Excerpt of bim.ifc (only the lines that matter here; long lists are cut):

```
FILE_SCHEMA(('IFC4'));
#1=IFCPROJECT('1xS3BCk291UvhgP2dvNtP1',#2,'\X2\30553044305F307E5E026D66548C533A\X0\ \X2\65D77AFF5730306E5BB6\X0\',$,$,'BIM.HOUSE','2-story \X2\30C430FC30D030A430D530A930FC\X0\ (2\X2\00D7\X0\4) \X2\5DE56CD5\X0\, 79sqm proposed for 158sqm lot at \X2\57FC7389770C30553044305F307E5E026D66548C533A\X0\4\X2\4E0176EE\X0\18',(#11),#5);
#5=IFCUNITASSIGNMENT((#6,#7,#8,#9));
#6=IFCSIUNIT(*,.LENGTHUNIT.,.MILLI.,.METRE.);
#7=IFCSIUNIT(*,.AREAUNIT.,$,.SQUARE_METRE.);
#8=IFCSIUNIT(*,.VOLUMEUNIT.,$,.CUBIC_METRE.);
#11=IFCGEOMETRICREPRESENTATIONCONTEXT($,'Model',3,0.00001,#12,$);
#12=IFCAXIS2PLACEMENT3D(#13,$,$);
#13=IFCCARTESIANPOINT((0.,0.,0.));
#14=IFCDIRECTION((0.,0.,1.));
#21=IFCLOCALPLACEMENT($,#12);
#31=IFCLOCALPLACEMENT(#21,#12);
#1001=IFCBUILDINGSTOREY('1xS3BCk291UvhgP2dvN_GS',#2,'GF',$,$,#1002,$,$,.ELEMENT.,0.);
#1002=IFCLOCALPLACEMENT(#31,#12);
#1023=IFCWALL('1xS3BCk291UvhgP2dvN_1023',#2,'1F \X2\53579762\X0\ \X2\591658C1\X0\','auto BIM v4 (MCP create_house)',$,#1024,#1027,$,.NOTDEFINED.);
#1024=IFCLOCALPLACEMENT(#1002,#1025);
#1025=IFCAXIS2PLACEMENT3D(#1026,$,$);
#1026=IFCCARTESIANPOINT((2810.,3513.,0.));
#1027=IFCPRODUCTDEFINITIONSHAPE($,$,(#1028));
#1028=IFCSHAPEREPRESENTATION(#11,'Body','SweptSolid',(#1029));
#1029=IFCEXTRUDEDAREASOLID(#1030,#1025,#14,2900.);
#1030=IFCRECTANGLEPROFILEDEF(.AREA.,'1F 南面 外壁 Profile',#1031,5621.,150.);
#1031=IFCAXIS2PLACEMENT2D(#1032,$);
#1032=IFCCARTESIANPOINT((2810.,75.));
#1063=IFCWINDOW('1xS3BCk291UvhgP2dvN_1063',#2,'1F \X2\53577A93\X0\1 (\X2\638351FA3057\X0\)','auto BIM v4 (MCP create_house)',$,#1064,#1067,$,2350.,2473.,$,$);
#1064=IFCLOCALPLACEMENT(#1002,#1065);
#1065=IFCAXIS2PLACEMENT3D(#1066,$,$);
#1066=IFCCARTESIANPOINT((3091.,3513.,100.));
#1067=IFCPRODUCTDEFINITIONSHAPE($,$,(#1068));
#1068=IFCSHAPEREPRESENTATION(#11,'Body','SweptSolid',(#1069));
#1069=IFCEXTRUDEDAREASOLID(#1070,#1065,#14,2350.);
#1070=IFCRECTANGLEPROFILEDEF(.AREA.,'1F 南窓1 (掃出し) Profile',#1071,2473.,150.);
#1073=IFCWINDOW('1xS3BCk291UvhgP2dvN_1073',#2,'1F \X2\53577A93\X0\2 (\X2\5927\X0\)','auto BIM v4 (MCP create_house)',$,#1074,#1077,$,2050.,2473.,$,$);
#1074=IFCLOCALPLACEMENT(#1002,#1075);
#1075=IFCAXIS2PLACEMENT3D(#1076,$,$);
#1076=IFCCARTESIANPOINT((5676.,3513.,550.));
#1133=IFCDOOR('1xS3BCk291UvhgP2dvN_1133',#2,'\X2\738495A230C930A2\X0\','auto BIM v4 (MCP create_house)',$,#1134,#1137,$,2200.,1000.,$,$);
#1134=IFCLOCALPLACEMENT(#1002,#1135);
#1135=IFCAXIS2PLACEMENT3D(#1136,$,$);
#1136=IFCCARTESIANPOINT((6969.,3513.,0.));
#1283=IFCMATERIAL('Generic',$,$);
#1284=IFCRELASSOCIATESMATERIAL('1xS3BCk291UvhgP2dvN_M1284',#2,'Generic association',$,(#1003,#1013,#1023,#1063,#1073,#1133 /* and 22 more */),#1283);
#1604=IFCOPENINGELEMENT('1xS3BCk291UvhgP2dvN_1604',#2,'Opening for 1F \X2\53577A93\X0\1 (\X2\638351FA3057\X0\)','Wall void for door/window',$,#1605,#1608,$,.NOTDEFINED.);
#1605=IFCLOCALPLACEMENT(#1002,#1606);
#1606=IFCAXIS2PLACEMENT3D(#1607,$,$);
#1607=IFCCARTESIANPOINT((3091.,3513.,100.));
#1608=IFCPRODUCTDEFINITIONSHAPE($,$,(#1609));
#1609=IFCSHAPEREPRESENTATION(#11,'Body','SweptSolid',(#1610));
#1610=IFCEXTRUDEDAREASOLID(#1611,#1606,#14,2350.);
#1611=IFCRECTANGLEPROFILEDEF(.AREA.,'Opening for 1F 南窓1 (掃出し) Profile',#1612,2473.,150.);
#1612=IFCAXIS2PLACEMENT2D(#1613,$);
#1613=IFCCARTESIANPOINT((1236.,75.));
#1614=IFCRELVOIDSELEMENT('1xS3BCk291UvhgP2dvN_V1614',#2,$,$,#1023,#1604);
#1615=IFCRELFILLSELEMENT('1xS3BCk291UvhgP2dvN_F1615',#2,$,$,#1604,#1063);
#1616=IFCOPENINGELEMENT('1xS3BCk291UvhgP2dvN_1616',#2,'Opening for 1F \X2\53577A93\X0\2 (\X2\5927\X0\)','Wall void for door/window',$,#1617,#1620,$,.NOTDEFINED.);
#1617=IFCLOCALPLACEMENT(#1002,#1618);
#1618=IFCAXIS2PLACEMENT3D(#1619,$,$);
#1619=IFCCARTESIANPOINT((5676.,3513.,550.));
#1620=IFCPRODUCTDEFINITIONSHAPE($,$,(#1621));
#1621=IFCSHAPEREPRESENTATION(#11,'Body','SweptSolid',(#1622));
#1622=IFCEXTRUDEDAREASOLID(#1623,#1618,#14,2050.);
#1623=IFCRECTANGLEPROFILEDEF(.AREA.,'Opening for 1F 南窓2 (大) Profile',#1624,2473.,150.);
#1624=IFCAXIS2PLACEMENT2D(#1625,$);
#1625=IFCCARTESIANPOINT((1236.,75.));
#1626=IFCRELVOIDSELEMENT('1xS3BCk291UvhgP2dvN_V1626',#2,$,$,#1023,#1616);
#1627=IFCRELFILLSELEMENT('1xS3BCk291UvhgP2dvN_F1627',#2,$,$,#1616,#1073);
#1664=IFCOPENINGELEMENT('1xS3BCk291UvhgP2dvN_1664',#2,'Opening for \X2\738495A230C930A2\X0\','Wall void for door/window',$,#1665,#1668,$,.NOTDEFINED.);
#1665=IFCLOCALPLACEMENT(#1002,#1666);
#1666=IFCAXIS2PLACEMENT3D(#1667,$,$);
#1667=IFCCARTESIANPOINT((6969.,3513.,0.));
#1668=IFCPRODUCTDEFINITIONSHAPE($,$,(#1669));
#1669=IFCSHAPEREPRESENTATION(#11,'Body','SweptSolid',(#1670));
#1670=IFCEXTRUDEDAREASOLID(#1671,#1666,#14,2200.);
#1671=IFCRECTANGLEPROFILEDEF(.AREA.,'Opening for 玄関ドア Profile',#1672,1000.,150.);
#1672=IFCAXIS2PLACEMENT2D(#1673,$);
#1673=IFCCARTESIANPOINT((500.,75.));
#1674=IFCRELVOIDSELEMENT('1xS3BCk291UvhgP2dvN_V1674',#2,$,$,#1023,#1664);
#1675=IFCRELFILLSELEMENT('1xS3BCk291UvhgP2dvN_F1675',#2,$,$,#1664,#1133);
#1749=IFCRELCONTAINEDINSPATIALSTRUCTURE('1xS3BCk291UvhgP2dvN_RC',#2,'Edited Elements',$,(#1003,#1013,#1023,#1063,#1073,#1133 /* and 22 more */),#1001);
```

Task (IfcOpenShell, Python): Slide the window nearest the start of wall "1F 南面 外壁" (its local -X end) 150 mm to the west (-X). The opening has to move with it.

```python
import ifcopenshell
import ifcopenshell.api.geometry
import ifcopenshell.util.placement
import ifcopenshell.util.unit

model = ifcopenshell.open("bim.ifc")
unit_scale = ifcopenshell.util.unit.calculate_unit_scale(model)

window = model.by_guid("1xS3BCk291UvhgP2dvN_1063")
opening = window.FillsVoids[0].RelatingOpeningElement
wall = opening.VoidsElements[0].RelatingBuildingElement

wall_matrix = ifcopenshell.util.placement.get_local_placement(wall.ObjectPlacement)
shift = wall_matrix[:3, 0] * -0.15 / unit_scale
before = ifcopenshell.util.placement.get_local_placement(window.ObjectPlacement)[:3, 3].copy()

# The window is not placed relative to its opening, so move both.
for product in (opening, window):
    matrix = ifcopenshell.util.placement.get_local_placement(product.ObjectPlacement)
    matrix[:3, 3] += shift
    ifcopenshell.api.geometry.edit_object_placement(model, product=product, matrix=matrix, is_si=False)

after = ifcopenshell.util.placement.get_local_placement(window.ObjectPlacement)[:3, 3]
print("window moved by", (after - before).round(3) + 0.0)

model.write("bim-out.ifc")
```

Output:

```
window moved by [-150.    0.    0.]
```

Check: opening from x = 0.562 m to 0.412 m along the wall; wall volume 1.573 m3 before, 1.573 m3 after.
